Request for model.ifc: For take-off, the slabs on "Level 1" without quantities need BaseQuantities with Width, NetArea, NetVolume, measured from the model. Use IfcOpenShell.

First a look at what the model holds.

```python
import ifcopenshell
import ifcopenshell.util.element
import ifcopenshell.util.unit

model = ifcopenshell.open("model.ifc")
print(model.schema)
for unit_type in ("LENGTHUNIT", "AREAUNIT", "VOLUMEUNIT"):
    print(unit_type, ifcopenshell.util.unit.calculate_unit_scale(model, unit_type))
storey = next(s for s in model.by_type("IfcBuildingStorey") if s.Name == "Level 1")
slabs = [e for e in ifcopenshell.util.element.get_decomposition(storey) if e.is_a("IfcSlab")]
for e in sorted(slabs, key=lambda e: e.id()):
    print(e.id(), e.is_a(), e.Name, list(ifcopenshell.util.element.get_psets(e, qtos_only=True)), sep=" | ")
```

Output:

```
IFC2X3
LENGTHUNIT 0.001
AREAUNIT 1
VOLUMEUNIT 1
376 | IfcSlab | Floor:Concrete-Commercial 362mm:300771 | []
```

```python
import ifcopenshell
import ifcopenshell.api.pset
import ifcopenshell.geom
import ifcopenshell.util.element
import ifcopenshell.util.shape
import ifcopenshell.util.unit

model = ifcopenshell.open("model.ifc")
unit_scale = ifcopenshell.util.unit.calculate_unit_scale(model)
area_scale = ifcopenshell.util.unit.calculate_unit_scale(model, "AREAUNIT")
volume_scale = ifcopenshell.util.unit.calculate_unit_scale(model, "VOLUMEUNIT")
settings = ifcopenshell.geom.settings()

storey = next(s for s in model.by_type("IfcBuildingStorey") if s.Name == "Level 1")
slabs = [e for e in ifcopenshell.util.element.get_decomposition(storey) if e.is_a("IfcSlab")]

for e in sorted(slabs, key=lambda e: e.id()):
    if ifcopenshell.util.element.get_psets(e, qtos_only=True, should_inherit=False):
        continue
    # Geometry comes back in metres, in the element's own axes.
    shape = ifcopenshell.geom.create_shape(settings, e)
    values = {
        "Width": ifcopenshell.util.shape.get_z(shape.geometry) / unit_scale,
        "NetArea": ifcopenshell.util.shape.get_footprint_area(shape.geometry) / area_scale,
        "NetVolume": ifcopenshell.util.shape.get_volume(shape.geometry) / volume_scale,
    }
    qto = ifcopenshell.api.pset.add_qto(model, product=e, name="BaseQuantities")
    ifcopenshell.api.pset.edit_qto(model, qto=qto, properties=values)
    print(e.id(), {k: round(v, 3) for k, v in values.items()})

model.write("model_edited.ifc")
```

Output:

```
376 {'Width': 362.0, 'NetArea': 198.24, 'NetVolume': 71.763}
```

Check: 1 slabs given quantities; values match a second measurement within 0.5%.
